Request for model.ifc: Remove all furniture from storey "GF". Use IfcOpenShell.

First a look at what the model holds.

```python
import ifcopenshell
import ifcopenshell.util.element

model = ifcopenshell.open("model.ifc")
print(model.schema)
storey = next(s for s in model.by_type("IfcBuildingStorey") if s.Name == "GF")
furniture = [e for e in ifcopenshell.util.element.get_decomposition(storey) if e.is_a("IfcFurnishingElement")]
seen = {}
for e in furniture:
    element_type = ifcopenshell.util.element.get_type(e)
    name = element_type.Name if element_type not in (None, e) else None
    seen[name] = seen.get(name, 0) + 1
for name, count in sorted(seen.items(), key=str):
    print(count, "x", name)
```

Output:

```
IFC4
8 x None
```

```python
import ifcopenshell
import ifcopenshell.api.root
import ifcopenshell.util.element

model = ifcopenshell.open("model.ifc")

storey = next(s for s in model.by_type("IfcBuildingStorey") if s.Name == "GF")
furniture = [e for e in ifcopenshell.util.element.get_decomposition(storey) if e.is_a("IfcFurnishingElement")]

for e in furniture:
    ifcopenshell.api.root.remove_product(model, product=e)
print(len(furniture), "removed")

model.write("model_edited.ifc")
```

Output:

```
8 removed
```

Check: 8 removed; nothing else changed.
